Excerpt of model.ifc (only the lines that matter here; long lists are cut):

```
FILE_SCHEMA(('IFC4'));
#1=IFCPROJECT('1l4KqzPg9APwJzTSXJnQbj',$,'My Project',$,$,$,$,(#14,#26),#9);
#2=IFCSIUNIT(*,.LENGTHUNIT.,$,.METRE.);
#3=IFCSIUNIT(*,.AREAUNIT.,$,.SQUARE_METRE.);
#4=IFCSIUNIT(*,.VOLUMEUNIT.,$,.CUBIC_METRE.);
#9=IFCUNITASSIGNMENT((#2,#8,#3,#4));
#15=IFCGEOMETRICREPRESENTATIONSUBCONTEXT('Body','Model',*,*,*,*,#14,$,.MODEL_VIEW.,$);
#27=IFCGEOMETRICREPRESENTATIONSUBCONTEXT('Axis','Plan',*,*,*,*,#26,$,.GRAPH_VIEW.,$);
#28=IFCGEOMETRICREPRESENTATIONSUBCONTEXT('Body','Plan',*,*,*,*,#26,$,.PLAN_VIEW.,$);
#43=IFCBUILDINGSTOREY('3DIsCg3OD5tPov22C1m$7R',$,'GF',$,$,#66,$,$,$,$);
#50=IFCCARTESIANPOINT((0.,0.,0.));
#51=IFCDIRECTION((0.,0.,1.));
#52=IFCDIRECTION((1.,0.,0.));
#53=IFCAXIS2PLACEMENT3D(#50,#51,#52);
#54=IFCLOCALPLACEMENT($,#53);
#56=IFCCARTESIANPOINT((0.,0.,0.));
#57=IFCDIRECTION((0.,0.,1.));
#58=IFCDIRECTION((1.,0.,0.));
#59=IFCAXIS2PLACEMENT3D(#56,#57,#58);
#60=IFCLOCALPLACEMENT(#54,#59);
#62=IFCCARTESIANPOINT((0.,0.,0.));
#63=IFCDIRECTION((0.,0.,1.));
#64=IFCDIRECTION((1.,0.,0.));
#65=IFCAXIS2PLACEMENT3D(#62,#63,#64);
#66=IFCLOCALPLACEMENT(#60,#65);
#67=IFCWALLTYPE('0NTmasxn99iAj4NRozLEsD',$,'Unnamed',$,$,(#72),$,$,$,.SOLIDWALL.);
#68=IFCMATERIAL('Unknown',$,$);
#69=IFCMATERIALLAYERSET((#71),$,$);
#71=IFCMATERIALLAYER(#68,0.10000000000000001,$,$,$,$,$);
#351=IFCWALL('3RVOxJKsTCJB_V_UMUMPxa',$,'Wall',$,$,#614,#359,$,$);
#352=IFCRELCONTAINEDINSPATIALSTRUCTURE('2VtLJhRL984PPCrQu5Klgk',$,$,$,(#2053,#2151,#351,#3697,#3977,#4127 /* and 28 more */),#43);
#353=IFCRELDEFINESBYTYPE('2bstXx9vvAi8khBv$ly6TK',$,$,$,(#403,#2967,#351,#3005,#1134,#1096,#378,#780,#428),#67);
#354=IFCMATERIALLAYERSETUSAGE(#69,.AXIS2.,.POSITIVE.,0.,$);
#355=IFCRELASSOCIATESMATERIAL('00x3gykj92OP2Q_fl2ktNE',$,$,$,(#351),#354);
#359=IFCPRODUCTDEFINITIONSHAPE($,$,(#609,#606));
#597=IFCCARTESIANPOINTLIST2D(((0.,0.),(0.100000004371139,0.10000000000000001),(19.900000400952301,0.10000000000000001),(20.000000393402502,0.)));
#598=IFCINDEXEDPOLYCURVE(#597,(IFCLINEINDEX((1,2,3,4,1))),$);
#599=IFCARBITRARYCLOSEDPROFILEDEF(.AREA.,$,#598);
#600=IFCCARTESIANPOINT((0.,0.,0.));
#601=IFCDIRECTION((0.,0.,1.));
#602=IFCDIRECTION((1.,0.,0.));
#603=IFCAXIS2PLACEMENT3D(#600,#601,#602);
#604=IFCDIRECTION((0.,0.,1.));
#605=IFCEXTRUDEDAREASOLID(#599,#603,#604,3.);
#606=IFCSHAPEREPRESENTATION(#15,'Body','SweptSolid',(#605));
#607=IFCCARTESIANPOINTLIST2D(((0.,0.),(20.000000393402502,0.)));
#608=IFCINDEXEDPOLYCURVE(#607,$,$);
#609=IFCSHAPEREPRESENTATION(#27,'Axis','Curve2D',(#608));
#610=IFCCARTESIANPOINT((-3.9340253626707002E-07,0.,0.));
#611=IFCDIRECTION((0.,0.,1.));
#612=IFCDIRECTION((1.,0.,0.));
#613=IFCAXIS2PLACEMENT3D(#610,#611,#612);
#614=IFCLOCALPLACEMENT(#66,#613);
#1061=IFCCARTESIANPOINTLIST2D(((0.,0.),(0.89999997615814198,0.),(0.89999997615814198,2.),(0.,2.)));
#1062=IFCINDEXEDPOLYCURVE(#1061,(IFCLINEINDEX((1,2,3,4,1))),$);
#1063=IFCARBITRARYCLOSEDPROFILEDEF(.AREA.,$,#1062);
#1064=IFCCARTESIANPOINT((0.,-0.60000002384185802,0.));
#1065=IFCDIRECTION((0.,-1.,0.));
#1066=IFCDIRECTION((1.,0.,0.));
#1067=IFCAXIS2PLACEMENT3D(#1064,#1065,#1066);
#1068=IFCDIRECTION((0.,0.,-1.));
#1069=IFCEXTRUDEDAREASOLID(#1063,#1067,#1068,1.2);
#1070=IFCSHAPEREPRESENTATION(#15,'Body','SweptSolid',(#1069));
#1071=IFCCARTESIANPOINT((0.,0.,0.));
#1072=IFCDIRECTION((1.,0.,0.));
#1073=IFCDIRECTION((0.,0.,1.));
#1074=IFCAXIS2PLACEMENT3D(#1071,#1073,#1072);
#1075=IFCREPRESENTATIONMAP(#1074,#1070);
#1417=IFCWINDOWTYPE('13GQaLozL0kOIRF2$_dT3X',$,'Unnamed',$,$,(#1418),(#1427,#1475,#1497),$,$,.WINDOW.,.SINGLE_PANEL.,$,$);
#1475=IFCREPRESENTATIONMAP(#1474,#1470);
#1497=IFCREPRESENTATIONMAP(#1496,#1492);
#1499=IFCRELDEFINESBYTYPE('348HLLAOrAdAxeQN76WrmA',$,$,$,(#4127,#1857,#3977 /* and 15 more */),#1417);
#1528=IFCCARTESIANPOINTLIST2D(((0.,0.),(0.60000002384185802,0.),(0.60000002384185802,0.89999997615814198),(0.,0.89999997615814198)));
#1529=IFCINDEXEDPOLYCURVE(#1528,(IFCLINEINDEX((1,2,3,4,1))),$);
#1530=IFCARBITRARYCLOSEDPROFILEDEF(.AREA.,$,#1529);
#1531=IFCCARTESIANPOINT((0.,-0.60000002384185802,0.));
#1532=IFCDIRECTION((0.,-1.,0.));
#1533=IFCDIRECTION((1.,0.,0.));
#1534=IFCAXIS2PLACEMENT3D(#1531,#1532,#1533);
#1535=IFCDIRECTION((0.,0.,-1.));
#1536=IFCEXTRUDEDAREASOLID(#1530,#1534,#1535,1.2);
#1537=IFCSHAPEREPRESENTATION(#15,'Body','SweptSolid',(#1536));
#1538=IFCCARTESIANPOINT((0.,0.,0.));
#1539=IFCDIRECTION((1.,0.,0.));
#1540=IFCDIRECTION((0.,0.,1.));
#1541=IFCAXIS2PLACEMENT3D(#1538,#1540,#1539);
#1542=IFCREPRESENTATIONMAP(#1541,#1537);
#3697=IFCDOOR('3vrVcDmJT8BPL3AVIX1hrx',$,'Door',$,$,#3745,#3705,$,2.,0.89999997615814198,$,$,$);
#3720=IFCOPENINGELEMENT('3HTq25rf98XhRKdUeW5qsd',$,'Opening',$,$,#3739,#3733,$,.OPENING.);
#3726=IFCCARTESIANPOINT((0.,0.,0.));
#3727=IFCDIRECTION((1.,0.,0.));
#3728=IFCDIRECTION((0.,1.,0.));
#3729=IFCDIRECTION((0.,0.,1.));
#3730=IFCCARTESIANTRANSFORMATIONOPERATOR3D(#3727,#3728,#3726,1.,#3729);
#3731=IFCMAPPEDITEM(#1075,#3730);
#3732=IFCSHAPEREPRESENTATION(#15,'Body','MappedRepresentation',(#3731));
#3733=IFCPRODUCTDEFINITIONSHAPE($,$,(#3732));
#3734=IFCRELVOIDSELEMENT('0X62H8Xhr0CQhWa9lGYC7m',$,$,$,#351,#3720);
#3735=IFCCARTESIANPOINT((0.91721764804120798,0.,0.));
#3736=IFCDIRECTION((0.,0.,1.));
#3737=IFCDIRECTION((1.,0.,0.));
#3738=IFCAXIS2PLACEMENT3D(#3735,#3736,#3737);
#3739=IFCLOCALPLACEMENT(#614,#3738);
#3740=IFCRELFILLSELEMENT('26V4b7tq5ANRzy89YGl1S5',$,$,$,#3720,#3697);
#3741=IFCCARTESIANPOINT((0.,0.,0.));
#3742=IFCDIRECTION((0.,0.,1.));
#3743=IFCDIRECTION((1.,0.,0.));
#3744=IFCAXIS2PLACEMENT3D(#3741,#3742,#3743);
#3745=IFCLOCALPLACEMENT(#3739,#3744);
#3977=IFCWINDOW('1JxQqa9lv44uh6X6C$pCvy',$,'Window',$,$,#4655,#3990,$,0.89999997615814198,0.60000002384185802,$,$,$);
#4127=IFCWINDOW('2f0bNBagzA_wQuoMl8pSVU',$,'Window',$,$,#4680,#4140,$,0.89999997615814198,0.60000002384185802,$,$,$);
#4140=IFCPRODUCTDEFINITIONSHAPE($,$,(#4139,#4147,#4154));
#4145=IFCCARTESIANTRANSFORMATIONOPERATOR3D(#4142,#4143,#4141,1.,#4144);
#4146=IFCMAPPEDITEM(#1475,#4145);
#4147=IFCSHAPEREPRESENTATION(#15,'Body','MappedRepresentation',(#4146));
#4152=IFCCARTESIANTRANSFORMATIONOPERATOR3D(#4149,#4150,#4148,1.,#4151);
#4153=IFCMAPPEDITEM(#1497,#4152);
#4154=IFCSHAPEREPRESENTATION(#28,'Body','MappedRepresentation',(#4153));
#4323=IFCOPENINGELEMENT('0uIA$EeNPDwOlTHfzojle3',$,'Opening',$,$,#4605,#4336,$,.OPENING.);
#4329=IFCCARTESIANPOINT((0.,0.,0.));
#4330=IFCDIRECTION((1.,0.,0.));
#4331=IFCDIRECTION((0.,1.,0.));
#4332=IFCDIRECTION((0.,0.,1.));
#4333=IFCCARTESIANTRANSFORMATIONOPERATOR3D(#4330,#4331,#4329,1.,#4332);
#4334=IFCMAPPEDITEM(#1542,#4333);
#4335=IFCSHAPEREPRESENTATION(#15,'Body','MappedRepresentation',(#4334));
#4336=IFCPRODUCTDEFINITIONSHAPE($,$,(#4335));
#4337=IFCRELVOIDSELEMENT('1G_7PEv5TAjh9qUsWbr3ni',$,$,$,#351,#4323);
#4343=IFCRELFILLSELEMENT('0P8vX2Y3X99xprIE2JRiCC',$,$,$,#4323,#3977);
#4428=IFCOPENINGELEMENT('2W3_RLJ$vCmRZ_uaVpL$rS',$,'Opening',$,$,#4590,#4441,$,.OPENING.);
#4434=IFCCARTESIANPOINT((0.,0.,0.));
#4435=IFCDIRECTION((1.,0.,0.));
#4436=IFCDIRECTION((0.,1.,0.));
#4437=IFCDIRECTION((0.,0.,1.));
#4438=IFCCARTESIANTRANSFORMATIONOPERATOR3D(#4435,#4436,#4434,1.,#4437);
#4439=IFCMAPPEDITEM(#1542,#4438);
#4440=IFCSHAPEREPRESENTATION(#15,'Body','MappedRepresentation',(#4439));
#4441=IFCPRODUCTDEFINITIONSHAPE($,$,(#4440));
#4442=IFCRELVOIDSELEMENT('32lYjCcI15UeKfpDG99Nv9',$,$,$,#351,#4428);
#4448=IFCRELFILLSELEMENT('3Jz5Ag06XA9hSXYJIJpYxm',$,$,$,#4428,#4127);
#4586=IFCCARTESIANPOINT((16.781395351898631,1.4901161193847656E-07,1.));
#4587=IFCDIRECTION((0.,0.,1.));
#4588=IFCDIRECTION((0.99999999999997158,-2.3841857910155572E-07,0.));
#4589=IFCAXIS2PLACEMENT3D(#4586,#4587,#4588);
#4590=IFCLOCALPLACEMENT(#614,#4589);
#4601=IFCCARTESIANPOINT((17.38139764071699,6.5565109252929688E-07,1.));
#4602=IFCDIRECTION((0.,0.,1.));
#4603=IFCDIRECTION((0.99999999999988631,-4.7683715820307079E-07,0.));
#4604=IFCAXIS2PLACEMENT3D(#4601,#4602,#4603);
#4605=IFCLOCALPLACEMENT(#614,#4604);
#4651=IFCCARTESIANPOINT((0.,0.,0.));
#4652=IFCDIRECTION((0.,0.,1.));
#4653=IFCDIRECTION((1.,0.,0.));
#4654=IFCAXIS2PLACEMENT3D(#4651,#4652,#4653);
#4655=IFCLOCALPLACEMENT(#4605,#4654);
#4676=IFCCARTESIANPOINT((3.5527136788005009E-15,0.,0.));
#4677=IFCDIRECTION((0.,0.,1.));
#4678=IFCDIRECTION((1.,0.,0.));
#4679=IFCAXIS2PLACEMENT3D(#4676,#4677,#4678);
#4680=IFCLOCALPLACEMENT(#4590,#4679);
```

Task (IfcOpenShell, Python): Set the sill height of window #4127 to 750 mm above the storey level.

```python
import numpy as np
import ifcopenshell
import ifcopenshell.api.geometry
import ifcopenshell.geom
import ifcopenshell.util.element
import ifcopenshell.util.placement
import ifcopenshell.util.shape
import ifcopenshell.util.unit

model = ifcopenshell.open("model.ifc")
unit_scale = ifcopenshell.util.unit.calculate_unit_scale(model)

window = model.by_guid("2f0bNBagzA_wQuoMl8pSVU")
opening = window.FillsVoids[0].RelatingOpeningElement
storey = ifcopenshell.util.element.get_container(window, ifc_class="IfcBuildingStorey")
level = ifcopenshell.util.placement.get_local_placement(storey.ObjectPlacement)[2, 3]

# The opening's origin need not be at the sill, so measure its lowest point.
shape = ifcopenshell.geom.create_shape(ifcopenshell.geom.settings(), opening)
bottom = ifcopenshell.util.shape.get_shape_bottom_elevation(shape, shape.geometry) / unit_scale
dz = level + 0.75 - bottom

shift = np.array([0.0, 0.0, dz])
# The window is placed relative to its opening, so it follows when the opening moves.
matrix = ifcopenshell.util.placement.get_local_placement(opening.ObjectPlacement)
matrix[:3, 3] += shift
ifcopenshell.api.geometry.edit_object_placement(
    model, product=opening, matrix=matrix, is_si=False, should_transform_children=True
)

print(f"moved by {dz * unit_scale:+.3f} m")

model.write("model_rev.ifc")
```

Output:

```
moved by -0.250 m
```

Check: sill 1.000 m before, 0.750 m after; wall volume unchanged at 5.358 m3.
